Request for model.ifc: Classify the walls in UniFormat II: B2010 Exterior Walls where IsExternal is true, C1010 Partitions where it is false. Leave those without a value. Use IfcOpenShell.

First a look at what the model holds.

```python
import ifcopenshell
import ifcopenshell.util.element

model = ifcopenshell.open("model.ifc")
print(model.schema)
print("classifications:", [c.Name for c in model.by_type("IfcClassification")])
values = [ifcopenshell.util.element.get_pset(e, "Pset_WallCommon", "IsExternal") for e in model.by_type("IfcWall")]
for value in (True, False, None):
    print("IsExternal", value, values.count(value))
```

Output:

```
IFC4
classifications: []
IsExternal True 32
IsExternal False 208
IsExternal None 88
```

```python
import ifcopenshell
import ifcopenshell.api.classification
import ifcopenshell.util.element

model = ifcopenshell.open("model.ifc")

system = ifcopenshell.api.classification.add_classification(model, classification="UniFormat II")

walls = model.by_type("IfcWall")
external = {e: ifcopenshell.util.element.get_pset(e, "Pset_WallCommon", "IsExternal") for e in walls}
for flag, code, name in ((True, "B2010", "Exterior Walls"), (False, "C1010", "Partitions")):
    products = [e for e in walls if external[e] is flag]
    ifcopenshell.api.classification.add_reference(
        model, products=products, classification=system, identification=code, name=name
    )
    print(code, len(products))

model.write("model_edited.ifc")
```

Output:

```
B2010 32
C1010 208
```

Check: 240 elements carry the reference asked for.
